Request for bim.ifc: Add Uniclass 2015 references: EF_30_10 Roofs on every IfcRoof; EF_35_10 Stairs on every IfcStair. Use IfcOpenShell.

First a look at what the model holds.

```python
import ifcopenshell

model = ifcopenshell.open("bim.ifc")
print(model.schema)
print("classifications:", [c.Name for c in model.by_type("IfcClassification")])
for ifc_class in ("IfcDoor", "IfcRoof", "IfcStair", "IfcWall", "IfcWindow"):
    print(ifc_class, len(model.by_type(ifc_class)))
```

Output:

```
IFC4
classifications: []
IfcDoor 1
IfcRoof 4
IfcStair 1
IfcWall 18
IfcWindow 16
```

```python
import ifcopenshell
import ifcopenshell.api.classification

model = ifcopenshell.open("bim.ifc")

system = ifcopenshell.api.classification.add_classification(model, classification="Uniclass 2015")

codes = {
    "IfcRoof": ("EF_30_10", "Roofs"),
    "IfcStair": ("EF_35_10", "Stairs"),
}
for ifc_class, (code, name) in codes.items():
    products = model.by_type(ifc_class)
    ifcopenshell.api.classification.add_reference(
        model, products=products, classification=system, identification=code, name=name
    )
    print(code, len(products))

model.write("bim_v2.ifc")
```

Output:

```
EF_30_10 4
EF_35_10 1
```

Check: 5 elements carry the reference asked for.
